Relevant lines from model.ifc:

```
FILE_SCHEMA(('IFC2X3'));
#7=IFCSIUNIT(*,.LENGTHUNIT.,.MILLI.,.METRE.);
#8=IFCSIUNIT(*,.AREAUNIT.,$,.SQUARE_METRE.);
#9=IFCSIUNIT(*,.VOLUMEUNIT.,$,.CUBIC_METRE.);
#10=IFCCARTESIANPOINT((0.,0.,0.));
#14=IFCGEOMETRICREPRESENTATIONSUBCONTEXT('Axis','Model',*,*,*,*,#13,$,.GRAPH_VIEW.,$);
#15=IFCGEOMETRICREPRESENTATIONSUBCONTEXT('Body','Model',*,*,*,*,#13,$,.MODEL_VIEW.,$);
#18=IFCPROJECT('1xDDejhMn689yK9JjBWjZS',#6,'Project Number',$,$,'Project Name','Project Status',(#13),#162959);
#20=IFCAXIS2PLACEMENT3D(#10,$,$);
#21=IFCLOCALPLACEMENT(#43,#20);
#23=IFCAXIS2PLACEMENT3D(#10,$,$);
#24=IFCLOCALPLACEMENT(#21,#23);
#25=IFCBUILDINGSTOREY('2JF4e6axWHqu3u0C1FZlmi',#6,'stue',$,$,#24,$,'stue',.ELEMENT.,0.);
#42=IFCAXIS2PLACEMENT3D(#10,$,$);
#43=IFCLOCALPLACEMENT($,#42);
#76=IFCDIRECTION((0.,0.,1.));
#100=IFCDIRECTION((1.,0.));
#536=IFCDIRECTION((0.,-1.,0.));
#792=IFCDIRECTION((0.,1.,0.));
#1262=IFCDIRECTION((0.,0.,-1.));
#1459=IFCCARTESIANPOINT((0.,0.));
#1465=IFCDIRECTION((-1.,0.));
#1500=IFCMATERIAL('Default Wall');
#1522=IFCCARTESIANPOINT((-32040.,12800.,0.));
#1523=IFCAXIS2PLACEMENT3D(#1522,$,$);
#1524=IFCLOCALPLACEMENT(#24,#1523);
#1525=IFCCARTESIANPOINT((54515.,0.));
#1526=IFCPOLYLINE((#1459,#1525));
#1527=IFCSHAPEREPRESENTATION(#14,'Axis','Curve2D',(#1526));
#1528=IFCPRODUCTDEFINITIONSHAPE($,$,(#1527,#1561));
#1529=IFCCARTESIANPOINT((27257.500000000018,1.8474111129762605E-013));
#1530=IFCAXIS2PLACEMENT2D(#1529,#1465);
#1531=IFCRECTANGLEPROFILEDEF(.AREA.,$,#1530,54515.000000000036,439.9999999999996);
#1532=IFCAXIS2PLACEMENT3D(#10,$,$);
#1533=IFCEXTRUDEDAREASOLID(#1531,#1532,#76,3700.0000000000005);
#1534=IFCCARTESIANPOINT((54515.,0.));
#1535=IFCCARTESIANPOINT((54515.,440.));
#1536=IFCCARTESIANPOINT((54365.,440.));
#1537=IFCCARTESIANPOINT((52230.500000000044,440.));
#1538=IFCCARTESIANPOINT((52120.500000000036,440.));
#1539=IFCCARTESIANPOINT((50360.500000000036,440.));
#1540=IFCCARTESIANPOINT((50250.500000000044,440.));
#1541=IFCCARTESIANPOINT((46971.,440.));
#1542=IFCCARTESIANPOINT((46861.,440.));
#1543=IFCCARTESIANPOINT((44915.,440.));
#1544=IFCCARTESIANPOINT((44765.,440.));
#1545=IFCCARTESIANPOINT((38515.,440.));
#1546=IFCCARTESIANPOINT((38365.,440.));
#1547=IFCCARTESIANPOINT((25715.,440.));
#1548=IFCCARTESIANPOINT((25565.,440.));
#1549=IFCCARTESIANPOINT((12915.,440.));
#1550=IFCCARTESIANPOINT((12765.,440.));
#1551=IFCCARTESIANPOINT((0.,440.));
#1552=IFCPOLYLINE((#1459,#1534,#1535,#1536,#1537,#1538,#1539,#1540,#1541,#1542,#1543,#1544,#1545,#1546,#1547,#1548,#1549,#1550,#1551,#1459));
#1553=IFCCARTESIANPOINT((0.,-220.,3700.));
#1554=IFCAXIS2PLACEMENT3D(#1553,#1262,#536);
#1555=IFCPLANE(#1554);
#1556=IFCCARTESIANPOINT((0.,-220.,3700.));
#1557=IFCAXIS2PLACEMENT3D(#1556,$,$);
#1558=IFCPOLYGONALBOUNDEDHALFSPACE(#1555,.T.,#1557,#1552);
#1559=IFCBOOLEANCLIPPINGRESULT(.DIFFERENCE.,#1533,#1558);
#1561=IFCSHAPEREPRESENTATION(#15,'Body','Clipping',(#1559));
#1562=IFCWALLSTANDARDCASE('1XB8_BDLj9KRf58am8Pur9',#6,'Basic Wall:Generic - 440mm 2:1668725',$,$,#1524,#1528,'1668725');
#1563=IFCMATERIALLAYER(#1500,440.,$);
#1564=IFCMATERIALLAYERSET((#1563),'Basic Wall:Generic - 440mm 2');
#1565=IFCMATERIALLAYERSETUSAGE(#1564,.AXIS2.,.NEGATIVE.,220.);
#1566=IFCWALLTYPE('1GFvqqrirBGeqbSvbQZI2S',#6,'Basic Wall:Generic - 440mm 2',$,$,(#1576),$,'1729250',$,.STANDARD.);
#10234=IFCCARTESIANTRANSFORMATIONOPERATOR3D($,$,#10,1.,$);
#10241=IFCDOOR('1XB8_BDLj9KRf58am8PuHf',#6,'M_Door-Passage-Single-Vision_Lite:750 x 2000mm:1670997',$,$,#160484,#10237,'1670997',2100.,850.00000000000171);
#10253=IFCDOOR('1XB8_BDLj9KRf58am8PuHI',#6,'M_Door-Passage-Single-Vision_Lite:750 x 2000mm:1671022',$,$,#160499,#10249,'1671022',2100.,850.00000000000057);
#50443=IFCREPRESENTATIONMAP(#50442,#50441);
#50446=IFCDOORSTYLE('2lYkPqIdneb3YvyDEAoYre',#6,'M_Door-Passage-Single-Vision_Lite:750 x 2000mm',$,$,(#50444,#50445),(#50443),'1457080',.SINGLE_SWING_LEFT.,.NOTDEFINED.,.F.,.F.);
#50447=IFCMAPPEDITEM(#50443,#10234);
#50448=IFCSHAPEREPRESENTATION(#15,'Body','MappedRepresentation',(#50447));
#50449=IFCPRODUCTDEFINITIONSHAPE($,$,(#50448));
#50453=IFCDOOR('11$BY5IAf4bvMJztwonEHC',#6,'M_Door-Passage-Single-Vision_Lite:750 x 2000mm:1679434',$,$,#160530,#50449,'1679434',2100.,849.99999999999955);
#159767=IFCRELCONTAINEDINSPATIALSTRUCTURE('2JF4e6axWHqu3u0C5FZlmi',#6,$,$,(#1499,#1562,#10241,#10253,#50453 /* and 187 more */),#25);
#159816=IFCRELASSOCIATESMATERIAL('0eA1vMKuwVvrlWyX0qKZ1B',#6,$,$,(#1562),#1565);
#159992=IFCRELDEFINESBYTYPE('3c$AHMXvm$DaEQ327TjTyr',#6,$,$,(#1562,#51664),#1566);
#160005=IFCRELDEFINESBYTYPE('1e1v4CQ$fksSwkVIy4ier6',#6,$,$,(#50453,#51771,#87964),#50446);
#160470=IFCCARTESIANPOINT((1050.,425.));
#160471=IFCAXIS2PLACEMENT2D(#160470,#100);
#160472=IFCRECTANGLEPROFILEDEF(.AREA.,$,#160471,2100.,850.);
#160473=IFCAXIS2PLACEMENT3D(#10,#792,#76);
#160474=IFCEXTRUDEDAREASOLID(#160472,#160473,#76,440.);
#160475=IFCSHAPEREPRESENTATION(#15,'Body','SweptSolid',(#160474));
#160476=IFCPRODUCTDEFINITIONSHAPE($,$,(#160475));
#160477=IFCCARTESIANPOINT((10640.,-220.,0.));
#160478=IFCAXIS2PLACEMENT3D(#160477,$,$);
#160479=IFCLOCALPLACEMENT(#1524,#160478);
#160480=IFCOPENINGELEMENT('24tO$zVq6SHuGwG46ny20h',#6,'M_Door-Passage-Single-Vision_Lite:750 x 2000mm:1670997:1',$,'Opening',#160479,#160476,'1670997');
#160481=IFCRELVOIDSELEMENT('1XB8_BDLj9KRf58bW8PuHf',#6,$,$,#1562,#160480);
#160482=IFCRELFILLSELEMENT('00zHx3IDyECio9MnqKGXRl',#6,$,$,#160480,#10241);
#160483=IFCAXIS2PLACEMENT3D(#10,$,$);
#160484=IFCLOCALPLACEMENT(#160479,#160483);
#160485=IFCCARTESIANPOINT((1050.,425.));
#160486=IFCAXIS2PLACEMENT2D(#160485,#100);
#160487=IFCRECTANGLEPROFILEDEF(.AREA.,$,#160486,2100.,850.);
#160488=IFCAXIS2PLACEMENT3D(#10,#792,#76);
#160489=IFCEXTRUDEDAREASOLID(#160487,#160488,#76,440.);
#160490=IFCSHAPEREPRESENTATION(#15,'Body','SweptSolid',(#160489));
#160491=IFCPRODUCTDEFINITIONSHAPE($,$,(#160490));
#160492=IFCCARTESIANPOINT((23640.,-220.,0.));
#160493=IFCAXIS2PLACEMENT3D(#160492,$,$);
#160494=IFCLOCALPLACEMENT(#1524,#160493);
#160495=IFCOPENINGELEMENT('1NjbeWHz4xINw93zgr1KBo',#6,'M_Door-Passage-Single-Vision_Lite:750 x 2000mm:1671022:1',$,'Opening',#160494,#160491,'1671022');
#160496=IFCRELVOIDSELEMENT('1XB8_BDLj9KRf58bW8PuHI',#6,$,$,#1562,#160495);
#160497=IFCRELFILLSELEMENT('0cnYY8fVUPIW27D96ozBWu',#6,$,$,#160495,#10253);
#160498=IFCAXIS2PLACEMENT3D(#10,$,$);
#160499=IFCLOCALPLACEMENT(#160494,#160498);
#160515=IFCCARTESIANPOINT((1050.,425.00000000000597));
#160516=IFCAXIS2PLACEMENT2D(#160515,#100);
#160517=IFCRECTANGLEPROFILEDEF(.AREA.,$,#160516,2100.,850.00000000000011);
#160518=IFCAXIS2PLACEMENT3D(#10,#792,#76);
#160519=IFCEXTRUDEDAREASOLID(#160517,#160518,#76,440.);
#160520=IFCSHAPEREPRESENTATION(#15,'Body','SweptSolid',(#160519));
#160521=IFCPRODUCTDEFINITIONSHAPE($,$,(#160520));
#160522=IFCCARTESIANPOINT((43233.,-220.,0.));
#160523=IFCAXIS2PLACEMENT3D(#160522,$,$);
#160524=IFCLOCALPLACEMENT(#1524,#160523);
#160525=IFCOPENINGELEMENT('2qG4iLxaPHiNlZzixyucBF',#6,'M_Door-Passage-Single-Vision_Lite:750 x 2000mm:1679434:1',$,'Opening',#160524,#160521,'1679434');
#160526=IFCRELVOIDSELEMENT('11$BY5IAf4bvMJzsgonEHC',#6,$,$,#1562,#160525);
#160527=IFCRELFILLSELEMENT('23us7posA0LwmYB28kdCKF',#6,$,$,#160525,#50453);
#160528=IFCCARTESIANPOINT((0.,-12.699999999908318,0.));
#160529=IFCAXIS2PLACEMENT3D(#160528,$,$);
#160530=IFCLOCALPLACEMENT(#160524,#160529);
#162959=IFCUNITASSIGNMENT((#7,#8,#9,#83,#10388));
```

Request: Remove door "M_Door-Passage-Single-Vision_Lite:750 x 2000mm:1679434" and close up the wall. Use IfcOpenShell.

```python
import ifcopenshell
import ifcopenshell.api.feature
import ifcopenshell.api.root
import ifcopenshell.geom
import ifcopenshell.util.shape

model = ifcopenshell.open("model.ifc")
settings = ifcopenshell.geom.settings()


def volume(element):
    """Net volume in cubic metres, openings subtracted."""
    shape = ifcopenshell.geom.create_shape(settings, element)
    return ifcopenshell.util.shape.get_volume(shape.geometry)


door = model.by_guid("11$BY5IAf4bvMJztwonEHC")
opening = door.FillsVoids[0].RelatingOpeningElement
wall = opening.VoidsElements[0].RelatingBuildingElement
before = volume(wall)

ifcopenshell.api.root.remove_product(model, product=door)
ifcopenshell.api.feature.remove_feature(model, feature=opening)

after = volume(wall)

print(f"wall volume {before:.3f} -> {after:.3f} m3")

model.write("model_updated.ifc")
```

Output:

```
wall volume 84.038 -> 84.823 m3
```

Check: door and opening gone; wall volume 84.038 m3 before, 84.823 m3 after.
